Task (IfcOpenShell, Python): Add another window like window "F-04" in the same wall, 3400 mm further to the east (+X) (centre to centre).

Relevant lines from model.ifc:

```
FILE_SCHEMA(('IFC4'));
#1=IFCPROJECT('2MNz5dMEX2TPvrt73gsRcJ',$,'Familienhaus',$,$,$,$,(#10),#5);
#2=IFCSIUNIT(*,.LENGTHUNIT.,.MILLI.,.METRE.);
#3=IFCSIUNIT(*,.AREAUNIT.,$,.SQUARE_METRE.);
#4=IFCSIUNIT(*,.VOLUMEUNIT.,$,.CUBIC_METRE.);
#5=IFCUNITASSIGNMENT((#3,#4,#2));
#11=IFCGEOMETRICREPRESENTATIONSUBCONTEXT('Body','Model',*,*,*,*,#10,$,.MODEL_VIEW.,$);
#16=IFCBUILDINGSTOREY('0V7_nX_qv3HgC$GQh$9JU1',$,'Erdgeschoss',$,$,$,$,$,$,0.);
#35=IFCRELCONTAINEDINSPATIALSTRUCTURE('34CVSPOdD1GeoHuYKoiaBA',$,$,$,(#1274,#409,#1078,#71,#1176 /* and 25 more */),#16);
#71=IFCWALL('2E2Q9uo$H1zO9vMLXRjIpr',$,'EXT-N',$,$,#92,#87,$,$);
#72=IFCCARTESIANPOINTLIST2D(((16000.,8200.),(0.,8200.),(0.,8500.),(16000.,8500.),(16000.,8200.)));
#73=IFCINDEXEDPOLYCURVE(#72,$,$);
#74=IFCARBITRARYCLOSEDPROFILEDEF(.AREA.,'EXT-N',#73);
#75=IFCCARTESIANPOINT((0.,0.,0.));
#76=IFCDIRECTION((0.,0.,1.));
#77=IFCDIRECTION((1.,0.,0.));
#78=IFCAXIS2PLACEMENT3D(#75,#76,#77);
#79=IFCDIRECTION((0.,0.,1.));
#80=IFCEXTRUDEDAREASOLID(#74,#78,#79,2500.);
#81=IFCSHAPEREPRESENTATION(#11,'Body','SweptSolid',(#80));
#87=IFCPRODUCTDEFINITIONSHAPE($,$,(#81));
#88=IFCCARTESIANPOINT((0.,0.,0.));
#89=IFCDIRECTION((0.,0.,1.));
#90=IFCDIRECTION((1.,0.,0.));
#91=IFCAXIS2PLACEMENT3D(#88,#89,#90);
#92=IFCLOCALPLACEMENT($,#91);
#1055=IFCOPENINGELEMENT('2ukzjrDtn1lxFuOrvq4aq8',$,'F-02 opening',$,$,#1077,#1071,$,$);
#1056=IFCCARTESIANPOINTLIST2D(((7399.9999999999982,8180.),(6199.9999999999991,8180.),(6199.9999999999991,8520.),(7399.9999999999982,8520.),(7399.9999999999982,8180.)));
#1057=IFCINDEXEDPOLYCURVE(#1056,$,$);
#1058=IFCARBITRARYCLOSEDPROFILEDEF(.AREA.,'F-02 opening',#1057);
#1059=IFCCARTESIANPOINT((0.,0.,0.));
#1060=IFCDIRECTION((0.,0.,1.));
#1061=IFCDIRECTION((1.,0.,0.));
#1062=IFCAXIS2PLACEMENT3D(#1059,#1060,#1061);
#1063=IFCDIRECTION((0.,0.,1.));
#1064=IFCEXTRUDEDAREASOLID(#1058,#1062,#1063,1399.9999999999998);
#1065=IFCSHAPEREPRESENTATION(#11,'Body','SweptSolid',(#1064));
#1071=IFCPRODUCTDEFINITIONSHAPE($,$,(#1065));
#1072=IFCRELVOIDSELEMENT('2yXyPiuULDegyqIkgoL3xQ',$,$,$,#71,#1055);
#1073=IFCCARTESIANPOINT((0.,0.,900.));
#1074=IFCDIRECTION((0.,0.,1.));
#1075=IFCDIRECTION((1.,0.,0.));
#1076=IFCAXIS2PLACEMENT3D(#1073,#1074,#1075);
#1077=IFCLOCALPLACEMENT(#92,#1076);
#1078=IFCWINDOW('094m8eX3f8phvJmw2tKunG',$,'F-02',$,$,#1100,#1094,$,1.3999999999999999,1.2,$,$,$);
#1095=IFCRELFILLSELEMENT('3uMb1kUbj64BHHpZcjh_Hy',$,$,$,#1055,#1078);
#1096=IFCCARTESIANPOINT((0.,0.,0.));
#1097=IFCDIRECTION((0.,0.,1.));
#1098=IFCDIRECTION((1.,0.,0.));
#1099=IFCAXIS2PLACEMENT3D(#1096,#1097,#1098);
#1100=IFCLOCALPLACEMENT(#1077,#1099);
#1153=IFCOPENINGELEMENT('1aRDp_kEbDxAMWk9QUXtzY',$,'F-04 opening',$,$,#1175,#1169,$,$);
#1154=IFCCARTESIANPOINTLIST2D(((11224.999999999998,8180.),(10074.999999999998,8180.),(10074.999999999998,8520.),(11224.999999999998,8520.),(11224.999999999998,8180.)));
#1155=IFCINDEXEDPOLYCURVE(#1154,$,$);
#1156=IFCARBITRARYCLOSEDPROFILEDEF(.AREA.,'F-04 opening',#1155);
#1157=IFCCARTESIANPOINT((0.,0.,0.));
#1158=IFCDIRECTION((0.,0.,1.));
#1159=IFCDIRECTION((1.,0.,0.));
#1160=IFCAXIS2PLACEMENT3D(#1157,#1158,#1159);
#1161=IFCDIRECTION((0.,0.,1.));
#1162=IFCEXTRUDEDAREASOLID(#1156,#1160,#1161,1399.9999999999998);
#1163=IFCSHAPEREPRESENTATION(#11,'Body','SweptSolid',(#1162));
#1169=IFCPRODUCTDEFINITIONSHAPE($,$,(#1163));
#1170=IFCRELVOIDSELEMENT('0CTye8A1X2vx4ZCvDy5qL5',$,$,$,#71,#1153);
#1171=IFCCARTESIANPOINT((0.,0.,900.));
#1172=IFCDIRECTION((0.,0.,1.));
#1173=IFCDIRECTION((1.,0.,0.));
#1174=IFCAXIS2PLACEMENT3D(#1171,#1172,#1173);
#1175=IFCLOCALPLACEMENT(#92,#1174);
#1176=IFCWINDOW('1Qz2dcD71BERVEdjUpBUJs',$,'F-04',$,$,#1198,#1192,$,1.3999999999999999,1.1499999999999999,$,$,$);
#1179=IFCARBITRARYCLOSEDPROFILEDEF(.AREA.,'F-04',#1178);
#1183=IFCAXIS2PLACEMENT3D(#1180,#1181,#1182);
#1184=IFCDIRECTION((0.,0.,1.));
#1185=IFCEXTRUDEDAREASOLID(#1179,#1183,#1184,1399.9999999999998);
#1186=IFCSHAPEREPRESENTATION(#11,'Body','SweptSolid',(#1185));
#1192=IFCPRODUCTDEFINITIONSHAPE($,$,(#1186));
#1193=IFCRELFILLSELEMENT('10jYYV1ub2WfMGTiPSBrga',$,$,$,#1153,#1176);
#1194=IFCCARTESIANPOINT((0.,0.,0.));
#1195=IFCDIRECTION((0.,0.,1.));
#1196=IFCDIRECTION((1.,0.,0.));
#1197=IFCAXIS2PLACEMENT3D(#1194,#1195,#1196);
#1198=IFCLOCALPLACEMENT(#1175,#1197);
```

```python
import ifcopenshell
import ifcopenshell.api.feature
import ifcopenshell.api.geometry
import ifcopenshell.api.root
import ifcopenshell.geom
import ifcopenshell.util.element
import ifcopenshell.util.placement
import ifcopenshell.util.shape
import ifcopenshell.util.unit

model = ifcopenshell.open("model.ifc")
unit_scale = ifcopenshell.util.unit.calculate_unit_scale(model)
settings = ifcopenshell.geom.settings()


def volume(element):
    """Net volume in cubic metres, openings subtracted."""
    shape = ifcopenshell.geom.create_shape(settings, element)
    return ifcopenshell.util.shape.get_volume(shape.geometry)


window = model.by_guid("1Qz2dcD71BERVEdjUpBUJs")
opening = window.FillsVoids[0].RelatingOpeningElement
wall = opening.VoidsElements[0].RelatingBuildingElement
before = volume(wall)
shift = ifcopenshell.util.placement.get_local_placement(wall.ObjectPlacement)[:3, 0] * 3.4 / unit_scale

# copy_class copies the void relationship, type, container and properties, but no geometry.
new_opening = ifcopenshell.api.root.copy_class(model, product=opening)
new_opening.Representation = ifcopenshell.util.element.copy_deep(
    model, opening.Representation, exclude=["IfcGeometricRepresentationContext", "IfcRepresentationMap"]
)
new_window = ifcopenshell.api.root.copy_class(model, product=window)
new_window.Representation = ifcopenshell.util.element.copy_deep(
    model, window.Representation, exclude=["IfcGeometricRepresentationContext", "IfcRepresentationMap"]
)
ifcopenshell.api.feature.add_filling(model, opening=new_opening, element=new_window)

for old, new in ((opening, new_opening), (window, new_window)):
    matrix = ifcopenshell.util.placement.get_local_placement(old.ObjectPlacement)
    matrix[:3, 3] += shift
    ifcopenshell.api.geometry.edit_object_placement(model, product=new, matrix=matrix, is_si=False)

after = volume(wall)

print(f"wall volume {before:.3f} -> {after:.3f} m3")

model.write("model_rev.ifc")
```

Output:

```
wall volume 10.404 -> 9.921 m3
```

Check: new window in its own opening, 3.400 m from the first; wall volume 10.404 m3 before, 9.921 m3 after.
